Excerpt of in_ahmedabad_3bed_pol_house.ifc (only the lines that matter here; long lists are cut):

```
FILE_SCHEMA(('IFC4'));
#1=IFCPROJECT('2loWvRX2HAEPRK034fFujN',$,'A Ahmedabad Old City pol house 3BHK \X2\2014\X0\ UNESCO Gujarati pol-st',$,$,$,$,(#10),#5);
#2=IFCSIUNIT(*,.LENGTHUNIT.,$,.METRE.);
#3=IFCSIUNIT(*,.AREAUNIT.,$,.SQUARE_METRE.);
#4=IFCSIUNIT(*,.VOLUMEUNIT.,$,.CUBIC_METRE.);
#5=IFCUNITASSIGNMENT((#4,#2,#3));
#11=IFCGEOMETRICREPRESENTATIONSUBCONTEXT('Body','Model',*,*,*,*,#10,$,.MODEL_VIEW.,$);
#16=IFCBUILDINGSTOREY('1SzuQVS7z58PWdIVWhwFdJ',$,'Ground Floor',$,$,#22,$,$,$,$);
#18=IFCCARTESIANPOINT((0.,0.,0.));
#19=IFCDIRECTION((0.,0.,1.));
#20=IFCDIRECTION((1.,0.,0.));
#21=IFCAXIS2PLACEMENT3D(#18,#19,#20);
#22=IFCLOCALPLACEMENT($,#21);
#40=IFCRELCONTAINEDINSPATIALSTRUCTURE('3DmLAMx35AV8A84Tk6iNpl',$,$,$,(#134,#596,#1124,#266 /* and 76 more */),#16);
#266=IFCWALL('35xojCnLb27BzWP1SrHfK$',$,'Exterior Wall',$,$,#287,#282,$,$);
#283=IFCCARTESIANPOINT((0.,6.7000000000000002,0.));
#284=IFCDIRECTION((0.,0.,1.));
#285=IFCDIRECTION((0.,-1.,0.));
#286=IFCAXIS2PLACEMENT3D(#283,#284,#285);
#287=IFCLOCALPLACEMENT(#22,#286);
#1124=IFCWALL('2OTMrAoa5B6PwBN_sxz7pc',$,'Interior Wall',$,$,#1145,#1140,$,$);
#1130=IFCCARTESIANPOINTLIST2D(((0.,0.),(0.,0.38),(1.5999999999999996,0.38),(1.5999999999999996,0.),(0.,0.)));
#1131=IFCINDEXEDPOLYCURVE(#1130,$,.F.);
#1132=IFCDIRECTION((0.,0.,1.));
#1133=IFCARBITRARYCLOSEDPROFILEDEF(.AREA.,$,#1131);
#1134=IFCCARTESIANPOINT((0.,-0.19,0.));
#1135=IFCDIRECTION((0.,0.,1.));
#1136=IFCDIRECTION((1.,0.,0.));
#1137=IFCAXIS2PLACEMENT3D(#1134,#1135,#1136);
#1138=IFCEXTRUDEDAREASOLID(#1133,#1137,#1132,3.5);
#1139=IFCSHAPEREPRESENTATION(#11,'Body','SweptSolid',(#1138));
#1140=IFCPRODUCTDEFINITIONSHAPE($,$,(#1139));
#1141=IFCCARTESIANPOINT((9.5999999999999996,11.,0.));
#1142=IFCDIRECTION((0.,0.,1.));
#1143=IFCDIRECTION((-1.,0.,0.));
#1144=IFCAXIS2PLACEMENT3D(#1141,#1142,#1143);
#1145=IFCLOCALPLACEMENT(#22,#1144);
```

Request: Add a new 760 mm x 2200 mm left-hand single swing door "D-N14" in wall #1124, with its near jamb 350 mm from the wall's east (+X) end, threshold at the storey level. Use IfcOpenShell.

```python
import numpy as np
import ifcopenshell
import ifcopenshell.api.feature
import ifcopenshell.api.geometry
import ifcopenshell.api.root
import ifcopenshell.api.spatial
import ifcopenshell.geom
import ifcopenshell.util.element
import ifcopenshell.util.placement
import ifcopenshell.util.representation
import ifcopenshell.util.shape
import ifcopenshell.util.unit

model = ifcopenshell.open("in_ahmedabad_3bed_pol_house.ifc")
unit_scale = ifcopenshell.util.unit.calculate_unit_scale(model)
settings = ifcopenshell.geom.settings()


def volume(element):
    """Net volume in cubic metres, openings subtracted."""
    shape = ifcopenshell.geom.create_shape(settings, element)
    return ifcopenshell.util.shape.get_volume(shape.geometry)


wall = model.by_guid("2OTMrAoa5B6PwBN_sxz7pc")
storey = ifcopenshell.util.element.get_container(wall, ifc_class="IfcBuildingStorey")
context = ifcopenshell.util.representation.get_context(model, "Model", "Body", "MODEL_VIEW")
before = volume(wall)

width, height, from_end, sill = 0.76, 2.2, 0.35, 0.0  # metres

# The wall runs along its own X axis, and the end named is its -X end.
wall_shape = ifcopenshell.geom.create_shape(settings, wall)
x, y, z = ifcopenshell.util.shape.get_vertices(wall_shape.geometry).T
start = x.min() + from_end
face, thickness = float(y.min()), float(y.max() - y.min())
wall_matrix = ifcopenshell.util.placement.get_local_placement(wall.ObjectPlacement)
level = ifcopenshell.util.placement.get_local_placement(storey.ObjectPlacement)[2, 3]


def in_wall(x, y):
    """Placement at x, y metres in the wall's axes, at sill height."""
    matrix = wall_matrix.copy()
    matrix[:, 3] = wall_matrix @ np.array([x / unit_scale, y / unit_scale, 0.0, 1.0])
    matrix[2, 3] = level + sill / unit_scale
    return matrix


# Opening: a box that overshoots both wall faces by 50 mm.
opening = ifcopenshell.api.root.create_entity(model, ifc_class="IfcOpeningElement", predefined_type="OPENING")
box = ifcopenshell.api.geometry.add_wall_representation(
    model, context=context, length=width, height=height, thickness=thickness + 0.1
)
ifcopenshell.api.geometry.assign_representation(model, product=opening, representation=box)
ifcopenshell.api.geometry.edit_object_placement(model, product=opening, matrix=in_wall(start, face - 0.05), is_si=False)
ifcopenshell.api.feature.add_feature(model, feature=opening, element=wall)

door = ifcopenshell.api.root.create_entity(model, ifc_class="IfcDoor", name="D-N14", predefined_type="DOOR")
door.OverallWidth, door.OverallHeight = width / unit_scale, height / unit_scale
door.OperationType = "SINGLE_SWING_LEFT"
body = ifcopenshell.api.geometry.add_door_representation(
    model,
    context=context,
    overall_width=door.OverallWidth,
    overall_height=door.OverallHeight,
    operation_type="SINGLE_SWING_LEFT",
    lining_properties={"LiningDepth": thickness / unit_scale, "ThresholdDepth": thickness / unit_scale},
)
ifcopenshell.api.geometry.assign_representation(model, product=door, representation=body)
ifcopenshell.api.spatial.assign_container(model, products=[door], relating_structure=storey)
ifcopenshell.api.feature.add_filling(model, opening=opening, element=door)

# The lining spans the wall, so the door starts at the wall face.
ifcopenshell.api.geometry.edit_object_placement(model, product=door, matrix=in_wall(start, face), is_si=False)

after = volume(wall)

print(f"wall volume {before:.3f} -> {after:.3f} m3")

model.write("in_ahmedabad_3bed_pol_house_rev.ifc")
```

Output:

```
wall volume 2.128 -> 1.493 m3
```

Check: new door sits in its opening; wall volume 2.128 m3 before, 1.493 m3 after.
